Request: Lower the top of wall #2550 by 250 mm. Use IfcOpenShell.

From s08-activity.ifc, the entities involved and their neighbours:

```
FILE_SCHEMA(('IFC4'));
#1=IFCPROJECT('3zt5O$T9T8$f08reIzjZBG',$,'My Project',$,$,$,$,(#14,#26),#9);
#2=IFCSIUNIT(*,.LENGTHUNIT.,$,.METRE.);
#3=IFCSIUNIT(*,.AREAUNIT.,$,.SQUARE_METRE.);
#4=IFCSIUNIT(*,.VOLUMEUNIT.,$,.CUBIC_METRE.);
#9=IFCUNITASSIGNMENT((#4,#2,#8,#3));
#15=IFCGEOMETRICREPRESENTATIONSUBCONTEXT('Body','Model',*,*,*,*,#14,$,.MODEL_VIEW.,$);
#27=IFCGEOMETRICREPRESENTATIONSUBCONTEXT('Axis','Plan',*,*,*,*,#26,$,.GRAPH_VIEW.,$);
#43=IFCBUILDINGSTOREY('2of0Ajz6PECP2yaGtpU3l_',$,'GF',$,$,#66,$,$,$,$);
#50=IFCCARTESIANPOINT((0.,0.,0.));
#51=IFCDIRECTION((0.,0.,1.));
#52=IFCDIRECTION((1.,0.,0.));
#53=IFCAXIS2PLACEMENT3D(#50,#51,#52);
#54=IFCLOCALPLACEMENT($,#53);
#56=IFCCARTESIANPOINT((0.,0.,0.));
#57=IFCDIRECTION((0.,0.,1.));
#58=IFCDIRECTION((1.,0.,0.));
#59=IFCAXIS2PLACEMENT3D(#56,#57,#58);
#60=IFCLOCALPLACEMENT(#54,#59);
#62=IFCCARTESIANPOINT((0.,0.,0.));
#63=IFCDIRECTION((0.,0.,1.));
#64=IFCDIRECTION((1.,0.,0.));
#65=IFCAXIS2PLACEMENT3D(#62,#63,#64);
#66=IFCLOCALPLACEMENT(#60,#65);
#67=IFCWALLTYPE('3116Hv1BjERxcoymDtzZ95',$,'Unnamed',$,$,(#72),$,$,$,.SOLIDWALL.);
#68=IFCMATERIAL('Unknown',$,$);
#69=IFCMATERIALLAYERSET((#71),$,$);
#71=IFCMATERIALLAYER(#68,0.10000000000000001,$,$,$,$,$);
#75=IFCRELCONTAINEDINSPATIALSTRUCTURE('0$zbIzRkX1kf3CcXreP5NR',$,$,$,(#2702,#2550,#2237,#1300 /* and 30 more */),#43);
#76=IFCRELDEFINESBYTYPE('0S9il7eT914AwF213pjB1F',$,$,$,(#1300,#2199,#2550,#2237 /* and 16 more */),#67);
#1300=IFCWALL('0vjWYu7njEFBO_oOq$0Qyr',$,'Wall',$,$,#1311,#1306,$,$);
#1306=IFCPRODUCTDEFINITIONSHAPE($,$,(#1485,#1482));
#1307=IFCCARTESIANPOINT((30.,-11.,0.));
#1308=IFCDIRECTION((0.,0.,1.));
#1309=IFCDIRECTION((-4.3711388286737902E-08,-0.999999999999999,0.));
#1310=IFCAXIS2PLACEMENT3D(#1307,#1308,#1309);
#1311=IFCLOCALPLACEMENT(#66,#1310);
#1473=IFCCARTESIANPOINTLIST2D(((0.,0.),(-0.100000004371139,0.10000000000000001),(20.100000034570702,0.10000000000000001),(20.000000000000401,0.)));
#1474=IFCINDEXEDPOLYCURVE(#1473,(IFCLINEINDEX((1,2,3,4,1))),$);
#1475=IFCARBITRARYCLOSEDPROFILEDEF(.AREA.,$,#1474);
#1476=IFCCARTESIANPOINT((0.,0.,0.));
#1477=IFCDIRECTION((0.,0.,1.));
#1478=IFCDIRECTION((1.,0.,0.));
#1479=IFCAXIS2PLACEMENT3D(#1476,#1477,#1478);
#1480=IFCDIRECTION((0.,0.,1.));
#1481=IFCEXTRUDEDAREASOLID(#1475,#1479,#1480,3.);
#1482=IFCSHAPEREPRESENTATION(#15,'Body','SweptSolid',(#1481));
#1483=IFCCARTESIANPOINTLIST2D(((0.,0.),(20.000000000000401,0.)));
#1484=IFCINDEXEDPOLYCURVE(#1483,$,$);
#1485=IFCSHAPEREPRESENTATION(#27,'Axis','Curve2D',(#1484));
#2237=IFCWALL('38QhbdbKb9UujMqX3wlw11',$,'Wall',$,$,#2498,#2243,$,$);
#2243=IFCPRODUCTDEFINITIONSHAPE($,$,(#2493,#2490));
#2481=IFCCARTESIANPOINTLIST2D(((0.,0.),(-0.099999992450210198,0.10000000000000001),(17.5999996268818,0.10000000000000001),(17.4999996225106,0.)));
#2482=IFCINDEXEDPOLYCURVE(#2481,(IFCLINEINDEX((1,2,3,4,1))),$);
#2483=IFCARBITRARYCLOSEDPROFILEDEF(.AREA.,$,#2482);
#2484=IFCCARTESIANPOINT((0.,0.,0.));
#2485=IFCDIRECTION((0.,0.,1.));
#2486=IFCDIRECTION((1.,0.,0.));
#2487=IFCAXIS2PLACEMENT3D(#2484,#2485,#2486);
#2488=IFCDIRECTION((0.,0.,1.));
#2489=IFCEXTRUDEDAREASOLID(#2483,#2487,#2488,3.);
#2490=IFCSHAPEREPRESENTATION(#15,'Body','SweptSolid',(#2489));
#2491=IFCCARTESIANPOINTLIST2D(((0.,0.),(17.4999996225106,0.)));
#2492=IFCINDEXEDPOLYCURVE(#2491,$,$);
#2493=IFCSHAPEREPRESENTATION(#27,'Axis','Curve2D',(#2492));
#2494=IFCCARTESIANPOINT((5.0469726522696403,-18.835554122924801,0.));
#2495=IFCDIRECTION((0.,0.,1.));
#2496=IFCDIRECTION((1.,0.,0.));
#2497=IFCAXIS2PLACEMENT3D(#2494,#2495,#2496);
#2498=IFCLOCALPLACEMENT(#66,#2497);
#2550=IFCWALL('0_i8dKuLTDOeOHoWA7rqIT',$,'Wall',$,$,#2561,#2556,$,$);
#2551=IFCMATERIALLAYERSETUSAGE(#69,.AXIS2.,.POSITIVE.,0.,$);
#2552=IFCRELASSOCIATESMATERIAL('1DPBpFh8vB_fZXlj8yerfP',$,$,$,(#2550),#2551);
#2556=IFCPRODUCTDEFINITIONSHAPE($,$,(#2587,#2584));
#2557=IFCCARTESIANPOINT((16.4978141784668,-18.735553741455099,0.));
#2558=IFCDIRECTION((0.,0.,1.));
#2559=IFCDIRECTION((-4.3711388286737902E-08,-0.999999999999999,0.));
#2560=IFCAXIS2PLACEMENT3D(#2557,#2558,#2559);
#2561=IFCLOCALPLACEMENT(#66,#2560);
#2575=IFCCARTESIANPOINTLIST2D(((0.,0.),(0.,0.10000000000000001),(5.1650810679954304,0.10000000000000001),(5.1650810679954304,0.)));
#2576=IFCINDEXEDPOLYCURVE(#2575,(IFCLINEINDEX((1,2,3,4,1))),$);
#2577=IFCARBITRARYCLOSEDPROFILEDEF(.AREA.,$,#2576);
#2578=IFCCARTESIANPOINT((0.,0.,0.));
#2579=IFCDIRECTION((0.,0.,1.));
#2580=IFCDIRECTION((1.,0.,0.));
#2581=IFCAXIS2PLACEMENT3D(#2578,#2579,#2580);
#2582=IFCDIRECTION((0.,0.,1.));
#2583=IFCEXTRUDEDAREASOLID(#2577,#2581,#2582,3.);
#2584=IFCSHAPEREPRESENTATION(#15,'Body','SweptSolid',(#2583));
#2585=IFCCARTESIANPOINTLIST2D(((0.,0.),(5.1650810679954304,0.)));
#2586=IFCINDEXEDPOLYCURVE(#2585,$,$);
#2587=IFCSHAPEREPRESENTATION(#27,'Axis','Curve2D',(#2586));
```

```python
import ifcopenshell
import ifcopenshell.geom
import ifcopenshell.util.representation
import ifcopenshell.util.shape
import ifcopenshell.util.unit

model = ifcopenshell.open("s08-activity.ifc")
unit_scale = ifcopenshell.util.unit.calculate_unit_scale(model)
settings = ifcopenshell.geom.settings()


def volume(element):
    """Net volume in cubic metres, openings subtracted."""
    shape = ifcopenshell.geom.create_shape(settings, element)
    return ifcopenshell.util.shape.get_volume(shape.geometry)


wall = model.by_guid("0_i8dKuLTDOeOHoWA7rqIT")
before = volume(wall)

body = ifcopenshell.util.representation.get_representation(wall, "Model", "Body")
solid = body.Items[0]
old_height = solid.Depth
solid.Depth -= 0.25 / unit_scale
after = volume(wall)

print(f"height {old_height:g} -> {solid.Depth:g}, volume {before:.3f} -> {after:.3f} m3")

model.write("s08-activity_rev.ifc")
```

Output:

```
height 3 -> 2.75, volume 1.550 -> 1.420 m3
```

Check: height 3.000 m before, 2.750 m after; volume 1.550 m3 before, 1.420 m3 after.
